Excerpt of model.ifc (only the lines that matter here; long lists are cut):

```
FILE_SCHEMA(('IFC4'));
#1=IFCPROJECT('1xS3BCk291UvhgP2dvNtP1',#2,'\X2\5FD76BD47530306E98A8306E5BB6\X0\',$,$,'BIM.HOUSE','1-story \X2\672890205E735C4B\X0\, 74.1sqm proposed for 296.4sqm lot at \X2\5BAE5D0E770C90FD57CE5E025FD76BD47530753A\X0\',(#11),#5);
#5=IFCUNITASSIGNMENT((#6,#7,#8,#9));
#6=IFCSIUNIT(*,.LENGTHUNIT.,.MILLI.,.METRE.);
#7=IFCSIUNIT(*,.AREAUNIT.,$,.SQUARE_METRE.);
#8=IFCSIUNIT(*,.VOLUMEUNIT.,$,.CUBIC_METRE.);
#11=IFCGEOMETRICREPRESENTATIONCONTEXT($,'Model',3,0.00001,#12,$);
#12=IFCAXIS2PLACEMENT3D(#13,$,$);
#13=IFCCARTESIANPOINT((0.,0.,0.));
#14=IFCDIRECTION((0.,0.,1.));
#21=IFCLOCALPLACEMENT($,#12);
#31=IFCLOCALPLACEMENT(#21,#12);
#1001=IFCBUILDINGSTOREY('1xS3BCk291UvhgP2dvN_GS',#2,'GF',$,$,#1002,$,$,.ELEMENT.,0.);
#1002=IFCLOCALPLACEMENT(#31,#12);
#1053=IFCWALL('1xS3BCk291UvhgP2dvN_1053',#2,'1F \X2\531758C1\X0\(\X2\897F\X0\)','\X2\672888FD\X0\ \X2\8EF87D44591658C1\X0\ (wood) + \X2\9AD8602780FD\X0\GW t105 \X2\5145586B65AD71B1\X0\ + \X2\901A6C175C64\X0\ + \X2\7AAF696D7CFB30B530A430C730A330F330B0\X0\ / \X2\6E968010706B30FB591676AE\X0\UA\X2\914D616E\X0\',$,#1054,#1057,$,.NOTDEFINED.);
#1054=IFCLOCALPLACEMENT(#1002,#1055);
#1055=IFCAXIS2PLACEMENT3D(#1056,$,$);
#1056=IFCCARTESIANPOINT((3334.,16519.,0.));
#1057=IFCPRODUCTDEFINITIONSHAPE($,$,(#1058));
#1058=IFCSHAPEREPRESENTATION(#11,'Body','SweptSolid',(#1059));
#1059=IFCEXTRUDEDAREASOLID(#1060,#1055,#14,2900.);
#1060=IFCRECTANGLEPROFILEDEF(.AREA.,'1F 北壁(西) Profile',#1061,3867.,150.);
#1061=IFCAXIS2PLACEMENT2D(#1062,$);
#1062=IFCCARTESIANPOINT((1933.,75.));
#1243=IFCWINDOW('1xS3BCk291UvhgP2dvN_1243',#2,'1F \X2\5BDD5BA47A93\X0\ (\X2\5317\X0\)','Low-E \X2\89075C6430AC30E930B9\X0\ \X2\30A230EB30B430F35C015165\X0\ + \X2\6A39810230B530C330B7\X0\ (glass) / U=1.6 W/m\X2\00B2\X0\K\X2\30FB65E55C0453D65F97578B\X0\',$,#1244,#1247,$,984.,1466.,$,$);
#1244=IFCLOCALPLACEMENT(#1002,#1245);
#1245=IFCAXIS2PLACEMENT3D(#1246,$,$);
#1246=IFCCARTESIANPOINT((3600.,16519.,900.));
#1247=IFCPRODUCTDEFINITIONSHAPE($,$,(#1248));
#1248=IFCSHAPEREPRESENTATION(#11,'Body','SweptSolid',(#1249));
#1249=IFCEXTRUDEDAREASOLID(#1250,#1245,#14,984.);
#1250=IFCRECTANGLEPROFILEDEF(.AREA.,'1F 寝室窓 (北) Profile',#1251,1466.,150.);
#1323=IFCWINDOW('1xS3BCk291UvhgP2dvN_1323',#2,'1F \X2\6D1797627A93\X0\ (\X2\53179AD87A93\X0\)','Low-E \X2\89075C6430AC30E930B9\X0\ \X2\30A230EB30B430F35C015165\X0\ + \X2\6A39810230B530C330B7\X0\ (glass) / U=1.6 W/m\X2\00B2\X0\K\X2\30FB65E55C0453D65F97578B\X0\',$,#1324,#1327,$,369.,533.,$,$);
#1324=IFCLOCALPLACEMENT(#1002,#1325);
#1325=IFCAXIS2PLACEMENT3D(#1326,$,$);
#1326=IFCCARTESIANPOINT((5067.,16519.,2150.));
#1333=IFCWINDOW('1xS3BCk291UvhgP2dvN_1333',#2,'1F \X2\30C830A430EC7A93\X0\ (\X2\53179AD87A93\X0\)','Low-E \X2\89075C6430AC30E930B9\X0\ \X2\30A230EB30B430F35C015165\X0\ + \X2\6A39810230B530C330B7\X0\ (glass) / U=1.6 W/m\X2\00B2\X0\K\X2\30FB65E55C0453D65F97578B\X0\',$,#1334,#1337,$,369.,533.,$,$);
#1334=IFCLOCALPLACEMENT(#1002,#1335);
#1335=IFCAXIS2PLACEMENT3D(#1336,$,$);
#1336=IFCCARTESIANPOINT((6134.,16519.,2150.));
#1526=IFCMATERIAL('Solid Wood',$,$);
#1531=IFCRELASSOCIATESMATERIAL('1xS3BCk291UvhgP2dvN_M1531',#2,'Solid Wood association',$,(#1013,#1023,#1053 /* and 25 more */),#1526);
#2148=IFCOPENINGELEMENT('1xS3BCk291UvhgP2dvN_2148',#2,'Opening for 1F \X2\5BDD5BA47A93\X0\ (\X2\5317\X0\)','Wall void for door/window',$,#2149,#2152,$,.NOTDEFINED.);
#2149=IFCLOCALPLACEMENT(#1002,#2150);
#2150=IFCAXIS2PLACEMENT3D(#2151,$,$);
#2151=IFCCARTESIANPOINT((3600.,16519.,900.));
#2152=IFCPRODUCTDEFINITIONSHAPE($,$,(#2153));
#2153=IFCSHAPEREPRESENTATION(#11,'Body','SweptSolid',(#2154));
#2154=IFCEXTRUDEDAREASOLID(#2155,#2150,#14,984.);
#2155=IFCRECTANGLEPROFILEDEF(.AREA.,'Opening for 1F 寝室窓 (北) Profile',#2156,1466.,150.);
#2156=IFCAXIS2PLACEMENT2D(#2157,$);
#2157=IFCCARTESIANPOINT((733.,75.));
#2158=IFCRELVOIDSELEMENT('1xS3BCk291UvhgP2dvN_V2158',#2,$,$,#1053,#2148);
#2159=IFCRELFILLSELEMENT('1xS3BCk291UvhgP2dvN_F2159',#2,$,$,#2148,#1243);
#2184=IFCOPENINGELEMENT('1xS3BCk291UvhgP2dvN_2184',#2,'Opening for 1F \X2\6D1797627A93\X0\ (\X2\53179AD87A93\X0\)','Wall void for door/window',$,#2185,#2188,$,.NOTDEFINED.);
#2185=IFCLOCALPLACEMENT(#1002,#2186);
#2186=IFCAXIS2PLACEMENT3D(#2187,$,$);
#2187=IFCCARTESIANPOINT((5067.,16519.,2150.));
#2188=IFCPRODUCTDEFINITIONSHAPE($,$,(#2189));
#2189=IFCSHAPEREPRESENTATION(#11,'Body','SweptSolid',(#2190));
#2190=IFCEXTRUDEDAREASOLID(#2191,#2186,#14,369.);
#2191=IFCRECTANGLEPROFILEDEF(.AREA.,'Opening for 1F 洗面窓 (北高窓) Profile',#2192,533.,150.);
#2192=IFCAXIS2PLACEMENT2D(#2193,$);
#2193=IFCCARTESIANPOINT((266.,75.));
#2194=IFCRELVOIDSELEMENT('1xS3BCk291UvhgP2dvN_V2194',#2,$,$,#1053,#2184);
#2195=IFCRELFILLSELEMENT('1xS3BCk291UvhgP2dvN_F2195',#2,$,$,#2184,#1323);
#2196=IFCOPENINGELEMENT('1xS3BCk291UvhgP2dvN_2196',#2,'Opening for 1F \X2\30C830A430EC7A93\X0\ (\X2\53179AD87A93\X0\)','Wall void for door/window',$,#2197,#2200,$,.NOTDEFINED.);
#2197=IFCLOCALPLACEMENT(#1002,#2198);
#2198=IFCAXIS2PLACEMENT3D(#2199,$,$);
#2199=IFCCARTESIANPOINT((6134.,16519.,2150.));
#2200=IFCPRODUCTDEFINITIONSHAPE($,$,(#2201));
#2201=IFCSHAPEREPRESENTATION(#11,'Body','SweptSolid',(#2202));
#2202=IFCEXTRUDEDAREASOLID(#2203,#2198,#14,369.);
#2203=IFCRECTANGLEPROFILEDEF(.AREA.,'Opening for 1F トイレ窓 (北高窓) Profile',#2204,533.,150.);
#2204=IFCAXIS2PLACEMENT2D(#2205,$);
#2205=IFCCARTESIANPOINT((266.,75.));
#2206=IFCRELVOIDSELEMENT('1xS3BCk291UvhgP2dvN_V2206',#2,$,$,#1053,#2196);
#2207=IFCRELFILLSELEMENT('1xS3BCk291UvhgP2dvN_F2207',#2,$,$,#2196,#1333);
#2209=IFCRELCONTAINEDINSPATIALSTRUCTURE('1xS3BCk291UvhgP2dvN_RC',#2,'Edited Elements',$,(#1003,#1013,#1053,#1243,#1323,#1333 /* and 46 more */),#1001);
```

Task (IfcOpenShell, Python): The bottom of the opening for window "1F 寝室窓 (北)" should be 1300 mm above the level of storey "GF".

```python
import numpy as np
import ifcopenshell
import ifcopenshell.api.geometry
import ifcopenshell.geom
import ifcopenshell.util.element
import ifcopenshell.util.placement
import ifcopenshell.util.shape
import ifcopenshell.util.unit

model = ifcopenshell.open("model.ifc")
unit_scale = ifcopenshell.util.unit.calculate_unit_scale(model)

window = model.by_id(1243)
opening = window.FillsVoids[0].RelatingOpeningElement
storey = ifcopenshell.util.element.get_container(window, ifc_class="IfcBuildingStorey")
level = ifcopenshell.util.placement.get_local_placement(storey.ObjectPlacement)[2, 3]

# The opening's origin need not be at the sill, so measure its lowest point.
shape = ifcopenshell.geom.create_shape(ifcopenshell.geom.settings(), opening)
bottom = ifcopenshell.util.shape.get_shape_bottom_elevation(shape, shape.geometry) / unit_scale
dz = level + 1.3 / unit_scale - bottom

shift = np.array([0.0, 0.0, dz])
# The window is not placed relative to its opening, so move both.
for product in (opening, window):
    matrix = ifcopenshell.util.placement.get_local_placement(product.ObjectPlacement)
    matrix[:3, 3] += shift
    ifcopenshell.api.geometry.edit_object_placement(model, product=product, matrix=matrix, is_si=False)

print(f"moved by {dz * unit_scale:+.3f} m")

model.write("model_updated.ifc")
```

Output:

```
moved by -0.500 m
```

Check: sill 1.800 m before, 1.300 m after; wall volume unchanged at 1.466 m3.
